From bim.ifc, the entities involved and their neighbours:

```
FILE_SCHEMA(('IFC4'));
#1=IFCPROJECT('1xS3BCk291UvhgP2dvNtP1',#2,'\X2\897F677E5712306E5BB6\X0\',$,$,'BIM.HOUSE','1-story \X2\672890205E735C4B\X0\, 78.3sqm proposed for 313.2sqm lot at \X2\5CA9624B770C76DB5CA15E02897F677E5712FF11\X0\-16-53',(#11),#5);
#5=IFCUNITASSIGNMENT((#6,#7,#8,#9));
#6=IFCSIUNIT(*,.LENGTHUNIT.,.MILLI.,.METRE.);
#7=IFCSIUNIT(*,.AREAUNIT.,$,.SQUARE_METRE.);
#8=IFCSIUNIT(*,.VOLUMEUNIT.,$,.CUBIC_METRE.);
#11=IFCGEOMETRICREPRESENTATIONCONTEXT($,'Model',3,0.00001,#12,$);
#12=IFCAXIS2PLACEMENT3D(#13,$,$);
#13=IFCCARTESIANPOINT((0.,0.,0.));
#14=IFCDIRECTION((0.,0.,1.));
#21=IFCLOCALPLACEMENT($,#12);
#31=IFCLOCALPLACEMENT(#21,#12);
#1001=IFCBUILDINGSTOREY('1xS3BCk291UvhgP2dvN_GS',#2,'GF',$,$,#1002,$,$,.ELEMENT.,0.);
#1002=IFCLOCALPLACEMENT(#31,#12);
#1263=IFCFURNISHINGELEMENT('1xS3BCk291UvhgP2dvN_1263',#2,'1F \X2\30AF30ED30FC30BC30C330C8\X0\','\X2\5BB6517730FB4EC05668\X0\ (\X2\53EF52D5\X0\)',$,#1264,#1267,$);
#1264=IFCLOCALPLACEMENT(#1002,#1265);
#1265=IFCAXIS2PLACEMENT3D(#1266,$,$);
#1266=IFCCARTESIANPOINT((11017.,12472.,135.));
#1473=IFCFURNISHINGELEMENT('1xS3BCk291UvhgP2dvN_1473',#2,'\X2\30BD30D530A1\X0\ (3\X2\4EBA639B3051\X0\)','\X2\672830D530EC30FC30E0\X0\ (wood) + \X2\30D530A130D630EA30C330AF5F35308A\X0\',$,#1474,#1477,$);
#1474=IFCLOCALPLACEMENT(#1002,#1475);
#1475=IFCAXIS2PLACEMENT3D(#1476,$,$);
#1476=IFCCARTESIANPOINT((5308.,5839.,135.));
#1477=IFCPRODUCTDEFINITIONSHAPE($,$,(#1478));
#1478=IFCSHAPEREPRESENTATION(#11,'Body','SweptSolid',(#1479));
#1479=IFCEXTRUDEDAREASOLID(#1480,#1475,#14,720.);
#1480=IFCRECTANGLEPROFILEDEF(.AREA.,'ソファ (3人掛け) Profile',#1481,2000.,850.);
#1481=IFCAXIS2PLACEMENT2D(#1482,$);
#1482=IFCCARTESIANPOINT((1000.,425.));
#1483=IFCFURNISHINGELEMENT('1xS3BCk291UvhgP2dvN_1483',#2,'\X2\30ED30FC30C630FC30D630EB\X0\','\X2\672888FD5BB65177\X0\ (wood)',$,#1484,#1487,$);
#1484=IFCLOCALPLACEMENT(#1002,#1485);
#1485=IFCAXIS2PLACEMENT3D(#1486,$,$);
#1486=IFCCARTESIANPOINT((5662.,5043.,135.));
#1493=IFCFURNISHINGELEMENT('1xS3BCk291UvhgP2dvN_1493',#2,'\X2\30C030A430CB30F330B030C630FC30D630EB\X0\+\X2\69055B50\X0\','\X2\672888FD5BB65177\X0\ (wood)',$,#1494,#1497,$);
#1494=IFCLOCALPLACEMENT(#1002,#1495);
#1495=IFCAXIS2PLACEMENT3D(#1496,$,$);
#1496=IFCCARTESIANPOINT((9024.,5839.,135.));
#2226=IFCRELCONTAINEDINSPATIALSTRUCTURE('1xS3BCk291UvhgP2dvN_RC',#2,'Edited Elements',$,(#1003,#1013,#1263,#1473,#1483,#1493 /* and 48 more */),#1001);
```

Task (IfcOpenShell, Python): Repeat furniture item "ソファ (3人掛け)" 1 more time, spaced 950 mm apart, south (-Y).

```python
import numpy as np
import ifcopenshell
import ifcopenshell.api.geometry
import ifcopenshell.api.root
import ifcopenshell.util.element
import ifcopenshell.util.placement

model = ifcopenshell.open("bim.ifc")


def reuse_history(source, copy):
    """copy_class also copies each property set's owner history, people and application; keep the originals."""
    for rel in copy.IsDefinedBy:
        if rel.is_a("IfcRelDefinesByProperties") and (history := rel.RelatingPropertyDefinition.OwnerHistory):
            rel.RelatingPropertyDefinition.OwnerHistory = source.OwnerHistory
            ifcopenshell.util.element.remove_deep2(model, history)


source = model.by_guid("1xS3BCk291UvhgP2dvN_1473")
base = ifcopenshell.util.placement.get_local_placement(source.ObjectPlacement)
step = np.array([0.0, -1.0, 0.0]) * 950.0

for i in range(1, 2):
    copy = ifcopenshell.api.root.copy_class(model, product=source)
    copy.Representation = ifcopenshell.util.element.copy_deep(
        model, source.Representation, exclude=["IfcGeometricRepresentationContext", "IfcRepresentationMap"]
    )
    reuse_history(source, copy)
    matrix = base.copy()
    matrix[:3, 3] += i * step
    print("added at", matrix[:3, 3].round(3) + 0.0)
    ifcopenshell.api.geometry.edit_object_placement(model, product=copy, matrix=matrix, is_si=False)

model.write("bim_rev.ifc")
```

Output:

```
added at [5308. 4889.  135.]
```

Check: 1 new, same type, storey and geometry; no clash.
